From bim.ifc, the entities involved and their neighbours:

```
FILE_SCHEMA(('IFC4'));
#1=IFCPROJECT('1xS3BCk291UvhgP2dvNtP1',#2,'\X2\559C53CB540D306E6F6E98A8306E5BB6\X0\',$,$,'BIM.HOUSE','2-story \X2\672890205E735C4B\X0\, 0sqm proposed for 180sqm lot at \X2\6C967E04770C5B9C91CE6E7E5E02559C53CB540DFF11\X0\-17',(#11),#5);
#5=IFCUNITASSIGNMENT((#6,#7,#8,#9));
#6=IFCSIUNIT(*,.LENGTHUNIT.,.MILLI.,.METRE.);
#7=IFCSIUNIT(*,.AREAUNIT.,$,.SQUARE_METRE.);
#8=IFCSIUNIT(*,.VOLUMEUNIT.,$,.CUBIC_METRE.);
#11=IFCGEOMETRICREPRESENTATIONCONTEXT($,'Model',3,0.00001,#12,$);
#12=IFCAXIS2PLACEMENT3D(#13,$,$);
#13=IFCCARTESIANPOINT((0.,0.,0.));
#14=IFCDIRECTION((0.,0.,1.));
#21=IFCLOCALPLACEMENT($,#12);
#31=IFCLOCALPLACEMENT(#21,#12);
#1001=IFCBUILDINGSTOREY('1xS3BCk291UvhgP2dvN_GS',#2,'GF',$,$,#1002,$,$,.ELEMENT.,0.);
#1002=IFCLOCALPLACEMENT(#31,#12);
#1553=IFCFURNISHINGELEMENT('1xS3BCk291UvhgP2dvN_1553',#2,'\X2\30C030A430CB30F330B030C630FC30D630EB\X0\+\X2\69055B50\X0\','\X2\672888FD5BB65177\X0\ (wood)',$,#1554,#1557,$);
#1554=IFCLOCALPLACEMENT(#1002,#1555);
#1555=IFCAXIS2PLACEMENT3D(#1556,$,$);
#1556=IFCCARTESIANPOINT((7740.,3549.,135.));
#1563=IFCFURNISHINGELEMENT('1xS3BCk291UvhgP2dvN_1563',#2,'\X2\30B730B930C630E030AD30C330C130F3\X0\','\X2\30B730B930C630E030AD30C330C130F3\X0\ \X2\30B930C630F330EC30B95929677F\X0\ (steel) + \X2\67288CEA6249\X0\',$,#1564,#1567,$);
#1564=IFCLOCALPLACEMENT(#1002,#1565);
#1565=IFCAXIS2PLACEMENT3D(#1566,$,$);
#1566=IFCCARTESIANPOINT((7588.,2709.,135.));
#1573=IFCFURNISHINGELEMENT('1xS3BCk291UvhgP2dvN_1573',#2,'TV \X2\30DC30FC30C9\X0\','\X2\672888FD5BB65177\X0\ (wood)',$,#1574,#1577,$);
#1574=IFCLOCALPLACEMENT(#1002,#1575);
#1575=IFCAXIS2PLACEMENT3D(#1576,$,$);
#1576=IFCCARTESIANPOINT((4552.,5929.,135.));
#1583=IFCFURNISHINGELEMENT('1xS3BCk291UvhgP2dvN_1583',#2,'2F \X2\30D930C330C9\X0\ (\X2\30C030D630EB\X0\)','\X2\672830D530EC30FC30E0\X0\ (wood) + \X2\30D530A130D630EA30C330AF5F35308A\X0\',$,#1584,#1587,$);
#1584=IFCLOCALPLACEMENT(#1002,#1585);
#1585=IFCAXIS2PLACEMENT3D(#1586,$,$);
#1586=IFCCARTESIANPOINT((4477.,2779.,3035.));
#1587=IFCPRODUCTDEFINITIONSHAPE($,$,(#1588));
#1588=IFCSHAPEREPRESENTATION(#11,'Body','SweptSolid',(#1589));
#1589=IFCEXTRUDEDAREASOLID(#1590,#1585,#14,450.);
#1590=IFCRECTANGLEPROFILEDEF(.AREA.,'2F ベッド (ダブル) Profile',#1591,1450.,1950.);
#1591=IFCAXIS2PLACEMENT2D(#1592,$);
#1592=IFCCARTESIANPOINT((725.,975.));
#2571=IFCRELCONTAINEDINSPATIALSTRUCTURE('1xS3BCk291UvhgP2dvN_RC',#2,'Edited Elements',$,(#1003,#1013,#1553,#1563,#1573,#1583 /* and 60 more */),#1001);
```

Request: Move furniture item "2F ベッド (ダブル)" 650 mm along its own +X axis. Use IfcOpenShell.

```python
import ifcopenshell
import ifcopenshell.api.geometry
import ifcopenshell.util.placement

model = ifcopenshell.open("bim.ifc")

item = model.by_guid("1xS3BCk291UvhgP2dvN_1583")
matrix = ifcopenshell.util.placement.get_local_placement(item.ObjectPlacement)
matrix[:3, 3] += matrix[:3, 0] * 650.0
ifcopenshell.api.geometry.edit_object_placement(model, product=item, matrix=matrix, is_si=False)

print(ifcopenshell.util.placement.get_local_placement(item.ObjectPlacement).round(3) + 0.0)

model.write("bim_edited.ifc")
```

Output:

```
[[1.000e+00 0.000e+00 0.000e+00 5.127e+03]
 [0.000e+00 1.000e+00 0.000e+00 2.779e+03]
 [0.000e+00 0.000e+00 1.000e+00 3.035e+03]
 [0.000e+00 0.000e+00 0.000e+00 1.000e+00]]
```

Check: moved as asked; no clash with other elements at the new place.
